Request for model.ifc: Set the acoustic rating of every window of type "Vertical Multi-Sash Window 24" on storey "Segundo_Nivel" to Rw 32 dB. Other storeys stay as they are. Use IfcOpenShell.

First a look at what the model holds.

```python
import ifcopenshell
import ifcopenshell.util.element

model = ifcopenshell.open("model.ifc")
print(model.schema)
storey = next(s for s in model.by_type("IfcBuildingStorey") if s.Name == "Segundo_Nivel")
windows = [e for e in ifcopenshell.util.element.get_decomposition(storey) if e.is_a("IfcWindow")]
seen = {}
for e in windows:
    element_type = ifcopenshell.util.element.get_type(e)
    key = (element_type.Name if element_type != e and element_type else None, ifcopenshell.util.element.get_pset(e, "Pset_WindowCommon", "AcousticRating"))
    seen[key] = seen.get(key, 0) + 1
for (name, value), count in sorted(seen.items(), key=str):
    print(count, "x", name, "|", value)
```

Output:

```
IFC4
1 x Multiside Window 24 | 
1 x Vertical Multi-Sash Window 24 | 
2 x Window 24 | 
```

```python
import ifcopenshell
import ifcopenshell.api.pset
import ifcopenshell.util.element

model = ifcopenshell.open("model.ifc")

storey = next(s for s in model.by_type("IfcBuildingStorey") if s.Name == "Segundo_Nivel")
windows = [e for e in ifcopenshell.util.element.get_decomposition(storey) if e.is_a("IfcWindow")]

count = 0
for e in windows:
    element_type = ifcopenshell.util.element.get_type(e)
    if element_type in (None, e) or element_type.Name != "Vertical Multi-Sash Window 24":
        continue
    # add_pset returns the element's existing set when there is one.
    pset = ifcopenshell.api.pset.add_pset(model, product=e, name="Pset_WindowCommon")
    ifcopenshell.api.pset.edit_pset(model, pset=pset, properties={"AcousticRating": "Rw 32 dB"})
    count += 1

print(count, "windows updated")

model.write("model_v2.ifc")
```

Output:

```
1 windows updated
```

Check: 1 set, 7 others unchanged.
